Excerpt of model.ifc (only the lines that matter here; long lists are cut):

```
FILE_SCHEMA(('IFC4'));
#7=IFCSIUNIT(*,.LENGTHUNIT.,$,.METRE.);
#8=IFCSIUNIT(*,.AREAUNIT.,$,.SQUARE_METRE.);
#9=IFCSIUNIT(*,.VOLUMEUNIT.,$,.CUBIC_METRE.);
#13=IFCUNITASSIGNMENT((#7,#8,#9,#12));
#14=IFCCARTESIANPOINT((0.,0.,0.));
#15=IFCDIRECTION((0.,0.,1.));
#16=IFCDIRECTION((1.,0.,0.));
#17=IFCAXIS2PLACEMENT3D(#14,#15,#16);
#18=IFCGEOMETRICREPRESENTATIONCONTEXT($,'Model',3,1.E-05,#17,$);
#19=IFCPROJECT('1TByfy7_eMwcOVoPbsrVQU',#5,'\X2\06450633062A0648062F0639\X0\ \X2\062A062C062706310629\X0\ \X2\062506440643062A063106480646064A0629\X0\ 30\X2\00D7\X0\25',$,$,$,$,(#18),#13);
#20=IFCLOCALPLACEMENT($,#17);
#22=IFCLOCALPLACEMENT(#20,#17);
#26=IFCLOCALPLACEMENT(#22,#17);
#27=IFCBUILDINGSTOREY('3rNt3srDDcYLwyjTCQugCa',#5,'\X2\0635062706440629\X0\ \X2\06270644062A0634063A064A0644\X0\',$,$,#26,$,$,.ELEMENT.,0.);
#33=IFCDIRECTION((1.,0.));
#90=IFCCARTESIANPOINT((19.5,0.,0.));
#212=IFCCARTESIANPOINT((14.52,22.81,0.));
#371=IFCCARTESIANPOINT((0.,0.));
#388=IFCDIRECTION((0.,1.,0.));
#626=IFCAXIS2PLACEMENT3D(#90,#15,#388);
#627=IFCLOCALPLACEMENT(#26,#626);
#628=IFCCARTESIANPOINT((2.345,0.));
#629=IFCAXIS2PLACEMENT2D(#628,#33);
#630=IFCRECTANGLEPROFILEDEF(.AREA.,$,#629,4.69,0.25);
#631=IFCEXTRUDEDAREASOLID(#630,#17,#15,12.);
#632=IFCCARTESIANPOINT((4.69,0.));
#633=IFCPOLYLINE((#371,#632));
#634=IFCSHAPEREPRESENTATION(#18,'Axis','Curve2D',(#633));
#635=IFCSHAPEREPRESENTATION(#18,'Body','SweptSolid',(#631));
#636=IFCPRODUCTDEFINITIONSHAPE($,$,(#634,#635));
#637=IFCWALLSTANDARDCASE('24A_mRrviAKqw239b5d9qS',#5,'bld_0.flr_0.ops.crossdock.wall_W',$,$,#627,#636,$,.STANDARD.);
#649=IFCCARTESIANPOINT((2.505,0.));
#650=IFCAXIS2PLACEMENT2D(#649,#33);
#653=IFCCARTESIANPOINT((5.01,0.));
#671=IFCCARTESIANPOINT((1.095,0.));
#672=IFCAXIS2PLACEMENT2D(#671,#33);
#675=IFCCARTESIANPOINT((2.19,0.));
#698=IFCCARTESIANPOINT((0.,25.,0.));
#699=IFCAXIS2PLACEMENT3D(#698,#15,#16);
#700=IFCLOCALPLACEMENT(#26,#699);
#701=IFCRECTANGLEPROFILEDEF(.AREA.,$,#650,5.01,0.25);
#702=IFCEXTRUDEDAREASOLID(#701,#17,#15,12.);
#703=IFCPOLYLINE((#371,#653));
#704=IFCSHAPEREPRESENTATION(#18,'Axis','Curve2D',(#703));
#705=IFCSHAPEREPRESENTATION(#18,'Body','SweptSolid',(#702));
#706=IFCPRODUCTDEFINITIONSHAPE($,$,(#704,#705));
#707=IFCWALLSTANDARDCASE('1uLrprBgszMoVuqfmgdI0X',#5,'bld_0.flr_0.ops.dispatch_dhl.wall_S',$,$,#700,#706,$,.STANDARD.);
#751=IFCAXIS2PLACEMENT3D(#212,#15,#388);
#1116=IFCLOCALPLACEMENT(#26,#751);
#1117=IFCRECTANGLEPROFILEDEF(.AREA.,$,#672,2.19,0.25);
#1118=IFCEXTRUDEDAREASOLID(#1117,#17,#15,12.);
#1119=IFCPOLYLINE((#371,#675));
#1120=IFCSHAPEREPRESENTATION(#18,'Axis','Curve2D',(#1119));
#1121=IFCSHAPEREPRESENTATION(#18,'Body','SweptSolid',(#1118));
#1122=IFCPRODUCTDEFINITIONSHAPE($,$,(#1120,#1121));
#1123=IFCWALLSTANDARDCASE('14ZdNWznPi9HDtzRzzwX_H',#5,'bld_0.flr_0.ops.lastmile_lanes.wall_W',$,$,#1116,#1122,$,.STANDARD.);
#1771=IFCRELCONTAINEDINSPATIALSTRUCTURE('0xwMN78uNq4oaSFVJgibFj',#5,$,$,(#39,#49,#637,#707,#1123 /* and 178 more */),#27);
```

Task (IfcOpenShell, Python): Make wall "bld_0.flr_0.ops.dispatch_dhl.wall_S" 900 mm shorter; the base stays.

```python
import ifcopenshell
import ifcopenshell.geom
import ifcopenshell.util.shape

model = ifcopenshell.open("model.ifc")
settings = ifcopenshell.geom.settings()


def volume(element):
    """Net volume in cubic metres, openings subtracted."""
    shape = ifcopenshell.geom.create_shape(settings, element)
    return ifcopenshell.util.shape.get_volume(shape.geometry)


wall = model.by_id(707)
before = volume(wall)

body = next(r for r in wall.Representation.Representations if r.RepresentationIdentifier == "Body")
solid = body.Items[0]
old_height = solid.Depth
solid.Depth -= 0.9
after = volume(wall)

print(f"height {old_height:g} -> {solid.Depth:g}, volume {before:.3f} -> {after:.3f} m3")

model.write("model-out.ifc")
```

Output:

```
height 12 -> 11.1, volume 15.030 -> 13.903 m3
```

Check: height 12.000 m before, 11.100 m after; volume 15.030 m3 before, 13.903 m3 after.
